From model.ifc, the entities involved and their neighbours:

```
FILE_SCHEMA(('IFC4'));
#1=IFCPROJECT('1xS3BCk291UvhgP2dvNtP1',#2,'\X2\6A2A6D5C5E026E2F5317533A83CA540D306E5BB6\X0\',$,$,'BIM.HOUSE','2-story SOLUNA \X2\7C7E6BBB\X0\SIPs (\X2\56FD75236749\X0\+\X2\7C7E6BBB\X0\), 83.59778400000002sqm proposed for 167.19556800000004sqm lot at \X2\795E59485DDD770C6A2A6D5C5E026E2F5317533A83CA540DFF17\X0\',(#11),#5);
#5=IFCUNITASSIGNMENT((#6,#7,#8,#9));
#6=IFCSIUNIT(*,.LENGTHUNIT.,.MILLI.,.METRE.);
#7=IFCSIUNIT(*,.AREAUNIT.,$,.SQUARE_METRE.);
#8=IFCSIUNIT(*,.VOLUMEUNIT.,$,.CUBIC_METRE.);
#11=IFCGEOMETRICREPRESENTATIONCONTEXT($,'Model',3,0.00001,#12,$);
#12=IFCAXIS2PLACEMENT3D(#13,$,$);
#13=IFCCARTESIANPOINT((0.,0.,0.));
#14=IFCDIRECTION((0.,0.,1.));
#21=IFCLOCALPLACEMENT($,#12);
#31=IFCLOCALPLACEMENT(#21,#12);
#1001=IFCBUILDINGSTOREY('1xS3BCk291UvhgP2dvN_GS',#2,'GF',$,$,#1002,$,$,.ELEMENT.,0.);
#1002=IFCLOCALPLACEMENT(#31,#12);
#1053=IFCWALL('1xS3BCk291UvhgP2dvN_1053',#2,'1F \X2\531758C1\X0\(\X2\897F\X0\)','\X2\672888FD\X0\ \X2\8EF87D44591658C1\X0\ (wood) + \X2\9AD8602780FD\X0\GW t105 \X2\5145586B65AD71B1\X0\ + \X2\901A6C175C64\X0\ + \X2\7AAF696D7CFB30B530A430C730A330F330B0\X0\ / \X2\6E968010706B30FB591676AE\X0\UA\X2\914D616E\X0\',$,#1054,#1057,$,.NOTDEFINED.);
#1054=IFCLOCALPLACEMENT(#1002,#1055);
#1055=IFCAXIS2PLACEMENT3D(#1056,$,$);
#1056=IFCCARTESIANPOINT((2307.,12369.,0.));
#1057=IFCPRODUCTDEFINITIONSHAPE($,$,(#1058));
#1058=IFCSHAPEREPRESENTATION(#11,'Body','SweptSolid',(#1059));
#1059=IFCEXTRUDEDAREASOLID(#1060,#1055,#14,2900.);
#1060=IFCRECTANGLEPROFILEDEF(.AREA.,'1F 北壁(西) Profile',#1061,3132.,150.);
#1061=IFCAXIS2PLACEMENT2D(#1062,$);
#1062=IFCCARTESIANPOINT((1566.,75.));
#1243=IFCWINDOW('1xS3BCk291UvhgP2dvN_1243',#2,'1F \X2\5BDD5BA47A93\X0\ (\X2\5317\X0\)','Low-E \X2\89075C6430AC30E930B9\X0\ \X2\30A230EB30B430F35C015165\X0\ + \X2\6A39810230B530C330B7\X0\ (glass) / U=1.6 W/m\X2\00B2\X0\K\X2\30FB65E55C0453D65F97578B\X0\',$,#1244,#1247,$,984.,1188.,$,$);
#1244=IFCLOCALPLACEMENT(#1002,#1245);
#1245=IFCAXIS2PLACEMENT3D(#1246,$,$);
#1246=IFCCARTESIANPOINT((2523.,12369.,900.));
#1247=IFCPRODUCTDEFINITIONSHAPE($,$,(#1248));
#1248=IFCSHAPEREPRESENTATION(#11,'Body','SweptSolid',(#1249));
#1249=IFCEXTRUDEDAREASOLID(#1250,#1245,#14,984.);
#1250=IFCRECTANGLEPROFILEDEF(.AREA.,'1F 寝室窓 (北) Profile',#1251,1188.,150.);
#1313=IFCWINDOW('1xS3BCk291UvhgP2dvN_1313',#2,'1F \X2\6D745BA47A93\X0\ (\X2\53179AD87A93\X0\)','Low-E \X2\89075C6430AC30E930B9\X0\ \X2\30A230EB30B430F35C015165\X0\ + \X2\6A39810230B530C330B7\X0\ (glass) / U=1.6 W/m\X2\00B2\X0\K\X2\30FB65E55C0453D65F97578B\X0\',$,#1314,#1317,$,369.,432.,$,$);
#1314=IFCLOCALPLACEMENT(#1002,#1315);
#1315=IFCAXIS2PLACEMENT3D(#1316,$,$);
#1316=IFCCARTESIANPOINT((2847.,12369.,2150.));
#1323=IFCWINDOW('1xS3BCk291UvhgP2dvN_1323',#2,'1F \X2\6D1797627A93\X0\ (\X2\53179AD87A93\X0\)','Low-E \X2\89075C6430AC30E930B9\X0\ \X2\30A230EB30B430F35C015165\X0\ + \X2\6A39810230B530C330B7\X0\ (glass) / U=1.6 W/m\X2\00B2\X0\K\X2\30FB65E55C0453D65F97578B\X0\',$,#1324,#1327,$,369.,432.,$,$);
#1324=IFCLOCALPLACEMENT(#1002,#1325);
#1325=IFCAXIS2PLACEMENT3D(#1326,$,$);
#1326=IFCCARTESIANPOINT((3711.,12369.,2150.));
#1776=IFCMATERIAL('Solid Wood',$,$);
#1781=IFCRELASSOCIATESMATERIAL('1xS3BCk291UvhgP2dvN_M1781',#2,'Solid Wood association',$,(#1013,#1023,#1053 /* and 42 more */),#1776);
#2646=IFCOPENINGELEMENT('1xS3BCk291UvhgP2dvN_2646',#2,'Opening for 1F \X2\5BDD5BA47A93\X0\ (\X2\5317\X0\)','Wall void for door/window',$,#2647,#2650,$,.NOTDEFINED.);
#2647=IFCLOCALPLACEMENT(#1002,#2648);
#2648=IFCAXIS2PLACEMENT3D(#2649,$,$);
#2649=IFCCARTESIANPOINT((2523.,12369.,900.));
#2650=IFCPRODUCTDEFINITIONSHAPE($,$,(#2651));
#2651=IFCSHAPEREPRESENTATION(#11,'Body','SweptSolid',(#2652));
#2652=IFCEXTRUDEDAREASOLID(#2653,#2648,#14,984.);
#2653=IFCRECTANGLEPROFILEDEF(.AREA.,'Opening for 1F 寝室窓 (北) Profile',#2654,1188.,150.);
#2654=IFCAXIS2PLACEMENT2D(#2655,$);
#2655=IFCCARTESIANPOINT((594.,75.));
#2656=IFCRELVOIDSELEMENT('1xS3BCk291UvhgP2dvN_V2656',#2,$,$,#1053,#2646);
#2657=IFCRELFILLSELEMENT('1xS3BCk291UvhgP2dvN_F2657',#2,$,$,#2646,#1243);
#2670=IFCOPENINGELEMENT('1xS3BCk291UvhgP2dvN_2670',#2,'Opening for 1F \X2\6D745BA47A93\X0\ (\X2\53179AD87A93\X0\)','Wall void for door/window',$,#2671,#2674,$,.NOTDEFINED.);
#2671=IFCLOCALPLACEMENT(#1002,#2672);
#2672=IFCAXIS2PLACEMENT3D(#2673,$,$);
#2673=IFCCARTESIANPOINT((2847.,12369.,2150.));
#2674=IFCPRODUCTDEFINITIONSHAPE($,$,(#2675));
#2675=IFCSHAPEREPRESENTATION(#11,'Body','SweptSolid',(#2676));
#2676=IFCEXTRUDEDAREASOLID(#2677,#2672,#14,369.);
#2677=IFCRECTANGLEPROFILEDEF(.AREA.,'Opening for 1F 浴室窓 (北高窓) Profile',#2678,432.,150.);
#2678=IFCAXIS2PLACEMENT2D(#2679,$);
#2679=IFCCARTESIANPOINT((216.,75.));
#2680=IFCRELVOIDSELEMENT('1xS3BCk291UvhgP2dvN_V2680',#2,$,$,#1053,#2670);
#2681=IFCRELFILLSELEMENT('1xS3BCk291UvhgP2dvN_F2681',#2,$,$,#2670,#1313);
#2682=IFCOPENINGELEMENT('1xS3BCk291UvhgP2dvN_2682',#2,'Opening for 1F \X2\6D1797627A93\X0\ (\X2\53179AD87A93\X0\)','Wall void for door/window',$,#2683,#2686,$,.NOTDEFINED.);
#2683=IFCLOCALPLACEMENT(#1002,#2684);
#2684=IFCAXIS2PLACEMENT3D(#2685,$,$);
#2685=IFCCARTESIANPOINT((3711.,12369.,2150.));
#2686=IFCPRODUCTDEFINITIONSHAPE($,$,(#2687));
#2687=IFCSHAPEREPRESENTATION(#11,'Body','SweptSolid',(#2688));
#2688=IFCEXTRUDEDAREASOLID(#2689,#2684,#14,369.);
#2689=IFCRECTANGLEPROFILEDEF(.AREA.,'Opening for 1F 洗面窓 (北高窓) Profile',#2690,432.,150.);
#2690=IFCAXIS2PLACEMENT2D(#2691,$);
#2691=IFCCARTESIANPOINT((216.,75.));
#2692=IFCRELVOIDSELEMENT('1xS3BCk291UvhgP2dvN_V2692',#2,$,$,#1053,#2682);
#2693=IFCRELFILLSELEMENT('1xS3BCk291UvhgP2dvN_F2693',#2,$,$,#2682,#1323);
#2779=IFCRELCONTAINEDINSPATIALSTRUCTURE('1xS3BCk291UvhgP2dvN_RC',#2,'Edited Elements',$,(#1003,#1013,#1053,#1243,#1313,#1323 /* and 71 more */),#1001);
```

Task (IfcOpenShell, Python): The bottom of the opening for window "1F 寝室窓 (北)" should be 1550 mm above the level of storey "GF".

```python
import numpy as np
import ifcopenshell
import ifcopenshell.api.geometry
import ifcopenshell.geom
import ifcopenshell.util.element
import ifcopenshell.util.placement
import ifcopenshell.util.shape
import ifcopenshell.util.unit

model = ifcopenshell.open("model.ifc")
unit_scale = ifcopenshell.util.unit.calculate_unit_scale(model)

window = model.by_guid("1xS3BCk291UvhgP2dvN_1243")
opening = window.FillsVoids[0].RelatingOpeningElement
storey = ifcopenshell.util.element.get_container(window, ifc_class="IfcBuildingStorey")
level = ifcopenshell.util.placement.get_local_placement(storey.ObjectPlacement)[2, 3]

# The opening's origin need not be at the sill, so measure its lowest point.
shape = ifcopenshell.geom.create_shape(ifcopenshell.geom.settings(), opening)
bottom = ifcopenshell.util.shape.get_shape_bottom_elevation(shape, shape.geometry) / unit_scale
dz = level + 1550.0 - bottom

shift = np.array([0.0, 0.0, dz])
# The window is not placed relative to its opening, so move both.
for product in (opening, window):
    matrix = ifcopenshell.util.placement.get_local_placement(product.ObjectPlacement)
    matrix[:3, 3] += shift
    ifcopenshell.api.geometry.edit_object_placement(model, product=product, matrix=matrix, is_si=False)

print(f"moved by {dz * unit_scale:+.3f} m")

model.write("model_v2.ifc")
```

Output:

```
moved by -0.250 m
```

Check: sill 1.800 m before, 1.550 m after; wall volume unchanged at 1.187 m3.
